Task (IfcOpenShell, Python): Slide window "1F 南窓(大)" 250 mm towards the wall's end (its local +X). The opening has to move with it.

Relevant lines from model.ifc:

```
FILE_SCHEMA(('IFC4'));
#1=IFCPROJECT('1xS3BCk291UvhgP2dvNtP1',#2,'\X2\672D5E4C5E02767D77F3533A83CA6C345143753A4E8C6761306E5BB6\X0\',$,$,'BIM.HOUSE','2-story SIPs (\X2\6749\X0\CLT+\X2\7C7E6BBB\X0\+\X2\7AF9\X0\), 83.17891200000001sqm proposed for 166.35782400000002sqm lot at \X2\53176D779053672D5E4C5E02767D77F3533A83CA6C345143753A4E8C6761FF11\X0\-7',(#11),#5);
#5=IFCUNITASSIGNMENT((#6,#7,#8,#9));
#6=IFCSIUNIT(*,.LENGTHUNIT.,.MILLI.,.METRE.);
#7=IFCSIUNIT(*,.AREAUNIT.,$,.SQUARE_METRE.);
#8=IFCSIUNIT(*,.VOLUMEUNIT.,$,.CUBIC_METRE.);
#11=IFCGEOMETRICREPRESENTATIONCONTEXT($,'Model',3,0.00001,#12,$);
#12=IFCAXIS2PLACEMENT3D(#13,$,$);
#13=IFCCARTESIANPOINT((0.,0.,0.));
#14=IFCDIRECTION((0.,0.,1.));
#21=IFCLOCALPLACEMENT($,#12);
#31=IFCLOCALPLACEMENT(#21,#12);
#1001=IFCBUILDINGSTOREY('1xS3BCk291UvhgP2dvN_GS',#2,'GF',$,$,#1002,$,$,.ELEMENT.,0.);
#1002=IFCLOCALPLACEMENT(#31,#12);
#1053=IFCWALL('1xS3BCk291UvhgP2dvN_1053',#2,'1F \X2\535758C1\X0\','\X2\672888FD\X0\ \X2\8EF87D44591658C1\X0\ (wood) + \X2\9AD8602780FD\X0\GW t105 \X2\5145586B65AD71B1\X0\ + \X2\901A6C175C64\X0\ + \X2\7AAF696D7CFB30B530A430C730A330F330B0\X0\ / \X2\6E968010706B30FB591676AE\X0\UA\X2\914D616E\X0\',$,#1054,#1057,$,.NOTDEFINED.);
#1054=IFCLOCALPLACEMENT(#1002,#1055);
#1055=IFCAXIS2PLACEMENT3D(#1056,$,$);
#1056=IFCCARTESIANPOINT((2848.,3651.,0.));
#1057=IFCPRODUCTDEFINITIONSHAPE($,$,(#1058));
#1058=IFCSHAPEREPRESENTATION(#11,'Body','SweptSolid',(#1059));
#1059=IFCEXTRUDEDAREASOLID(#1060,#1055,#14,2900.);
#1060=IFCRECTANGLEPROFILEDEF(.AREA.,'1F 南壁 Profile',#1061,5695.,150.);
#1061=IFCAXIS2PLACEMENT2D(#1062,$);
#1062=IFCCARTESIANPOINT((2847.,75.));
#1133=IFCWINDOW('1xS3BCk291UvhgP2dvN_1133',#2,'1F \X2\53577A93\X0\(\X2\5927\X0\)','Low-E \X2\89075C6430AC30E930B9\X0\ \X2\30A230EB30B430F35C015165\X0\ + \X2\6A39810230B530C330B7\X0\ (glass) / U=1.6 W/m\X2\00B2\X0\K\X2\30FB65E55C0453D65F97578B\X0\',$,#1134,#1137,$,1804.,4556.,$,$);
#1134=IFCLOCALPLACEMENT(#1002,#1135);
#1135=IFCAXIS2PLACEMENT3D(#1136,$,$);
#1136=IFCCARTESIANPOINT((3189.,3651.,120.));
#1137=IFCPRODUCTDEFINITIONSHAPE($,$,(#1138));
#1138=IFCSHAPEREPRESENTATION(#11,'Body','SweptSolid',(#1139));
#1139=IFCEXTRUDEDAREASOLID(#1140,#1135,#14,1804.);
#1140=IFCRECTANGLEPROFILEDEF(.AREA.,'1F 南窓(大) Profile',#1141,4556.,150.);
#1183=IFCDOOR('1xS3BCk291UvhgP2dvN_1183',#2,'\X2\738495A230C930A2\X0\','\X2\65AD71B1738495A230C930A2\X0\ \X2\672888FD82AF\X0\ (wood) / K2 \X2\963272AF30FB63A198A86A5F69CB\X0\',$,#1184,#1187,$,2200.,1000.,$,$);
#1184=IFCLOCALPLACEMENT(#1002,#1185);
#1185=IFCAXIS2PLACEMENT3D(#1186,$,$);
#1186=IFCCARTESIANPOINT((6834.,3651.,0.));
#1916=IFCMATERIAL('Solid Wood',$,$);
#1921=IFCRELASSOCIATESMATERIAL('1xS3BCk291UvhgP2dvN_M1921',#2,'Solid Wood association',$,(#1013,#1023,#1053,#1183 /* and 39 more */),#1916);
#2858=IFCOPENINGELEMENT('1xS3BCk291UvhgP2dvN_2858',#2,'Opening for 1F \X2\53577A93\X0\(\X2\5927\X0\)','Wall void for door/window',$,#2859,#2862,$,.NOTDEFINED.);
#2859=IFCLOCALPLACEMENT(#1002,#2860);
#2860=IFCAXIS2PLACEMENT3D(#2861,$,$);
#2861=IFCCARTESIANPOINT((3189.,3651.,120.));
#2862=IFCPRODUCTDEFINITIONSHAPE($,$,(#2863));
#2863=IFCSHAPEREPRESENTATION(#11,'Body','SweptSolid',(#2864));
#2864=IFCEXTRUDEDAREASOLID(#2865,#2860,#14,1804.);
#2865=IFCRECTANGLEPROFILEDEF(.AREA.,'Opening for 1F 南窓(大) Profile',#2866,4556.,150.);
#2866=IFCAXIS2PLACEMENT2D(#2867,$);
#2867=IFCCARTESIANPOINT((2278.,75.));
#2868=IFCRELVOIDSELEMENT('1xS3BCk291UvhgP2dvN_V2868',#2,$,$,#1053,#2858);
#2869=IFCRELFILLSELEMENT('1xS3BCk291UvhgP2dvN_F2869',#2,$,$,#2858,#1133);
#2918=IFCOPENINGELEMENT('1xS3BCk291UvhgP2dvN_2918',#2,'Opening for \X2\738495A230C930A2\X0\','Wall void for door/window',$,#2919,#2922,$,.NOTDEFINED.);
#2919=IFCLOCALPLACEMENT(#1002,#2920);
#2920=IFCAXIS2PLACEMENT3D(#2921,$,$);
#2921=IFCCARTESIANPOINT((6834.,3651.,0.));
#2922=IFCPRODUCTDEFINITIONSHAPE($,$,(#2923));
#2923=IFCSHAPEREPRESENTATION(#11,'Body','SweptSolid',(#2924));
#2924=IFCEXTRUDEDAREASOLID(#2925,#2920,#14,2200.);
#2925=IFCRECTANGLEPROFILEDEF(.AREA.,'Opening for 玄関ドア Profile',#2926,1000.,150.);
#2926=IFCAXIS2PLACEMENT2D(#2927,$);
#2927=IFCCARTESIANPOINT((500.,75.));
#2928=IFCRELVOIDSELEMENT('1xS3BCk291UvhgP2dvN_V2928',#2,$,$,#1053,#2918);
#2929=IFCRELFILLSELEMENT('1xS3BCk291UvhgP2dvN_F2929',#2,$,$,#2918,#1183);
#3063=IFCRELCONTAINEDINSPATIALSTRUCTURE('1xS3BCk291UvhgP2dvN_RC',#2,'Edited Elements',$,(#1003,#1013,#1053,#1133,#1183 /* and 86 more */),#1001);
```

```python
import ifcopenshell
import ifcopenshell.api.geometry
import ifcopenshell.util.placement
import ifcopenshell.util.unit

model = ifcopenshell.open("model.ifc")
unit_scale = ifcopenshell.util.unit.calculate_unit_scale(model)

window = model.by_guid("1xS3BCk291UvhgP2dvN_1133")
opening = window.FillsVoids[0].RelatingOpeningElement
wall = opening.VoidsElements[0].RelatingBuildingElement

wall_matrix = ifcopenshell.util.placement.get_local_placement(wall.ObjectPlacement)
shift = wall_matrix[:3, 0] * 0.25 / unit_scale
before = ifcopenshell.util.placement.get_local_placement(window.ObjectPlacement)[:3, 3].copy()

# The window is not placed relative to its opening, so move both.
for product in (opening, window):
    matrix = ifcopenshell.util.placement.get_local_placement(product.ObjectPlacement)
    matrix[:3, 3] += shift
    ifcopenshell.api.geometry.edit_object_placement(model, product=product, matrix=matrix, is_si=False)

after = ifcopenshell.util.placement.get_local_placement(window.ObjectPlacement)[:3, 3]
print("window moved by", (after - before).round(3) + 0.0)

model.write("model_edited.ifc")
```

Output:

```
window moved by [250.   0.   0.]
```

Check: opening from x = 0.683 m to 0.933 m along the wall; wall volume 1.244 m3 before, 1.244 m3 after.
